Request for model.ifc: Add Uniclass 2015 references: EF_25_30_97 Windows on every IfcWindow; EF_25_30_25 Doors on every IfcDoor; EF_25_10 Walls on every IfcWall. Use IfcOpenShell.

First a look at what the model holds.

```python
import ifcopenshell

model = ifcopenshell.open("model.ifc")
print(model.schema)
print("classifications:", [c.Name for c in model.by_type("IfcClassification")])
for ifc_class in ("IfcDoor", "IfcRoof", "IfcStair", "IfcWall", "IfcWindow"):
    print(ifc_class, len(model.by_type(ifc_class)))
```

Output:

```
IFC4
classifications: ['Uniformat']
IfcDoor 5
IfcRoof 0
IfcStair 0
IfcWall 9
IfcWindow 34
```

```python
import ifcopenshell
import ifcopenshell.api.classification

model = ifcopenshell.open("model.ifc")

system = ifcopenshell.api.classification.add_classification(model, classification="Uniclass 2015")

codes = {
    "IfcWindow": ("EF_25_30_97", "Windows"),
    "IfcDoor": ("EF_25_30_25", "Doors"),
    "IfcWall": ("EF_25_10", "Walls"),
}
for ifc_class, (code, name) in codes.items():
    products = model.by_type(ifc_class)
    ifcopenshell.api.classification.add_reference(
        model, products=products, classification=system, identification=code, name=name
    )
    print(code, len(products))

model.write("model_edited.ifc")
```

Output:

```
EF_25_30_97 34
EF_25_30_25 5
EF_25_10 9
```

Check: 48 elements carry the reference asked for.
